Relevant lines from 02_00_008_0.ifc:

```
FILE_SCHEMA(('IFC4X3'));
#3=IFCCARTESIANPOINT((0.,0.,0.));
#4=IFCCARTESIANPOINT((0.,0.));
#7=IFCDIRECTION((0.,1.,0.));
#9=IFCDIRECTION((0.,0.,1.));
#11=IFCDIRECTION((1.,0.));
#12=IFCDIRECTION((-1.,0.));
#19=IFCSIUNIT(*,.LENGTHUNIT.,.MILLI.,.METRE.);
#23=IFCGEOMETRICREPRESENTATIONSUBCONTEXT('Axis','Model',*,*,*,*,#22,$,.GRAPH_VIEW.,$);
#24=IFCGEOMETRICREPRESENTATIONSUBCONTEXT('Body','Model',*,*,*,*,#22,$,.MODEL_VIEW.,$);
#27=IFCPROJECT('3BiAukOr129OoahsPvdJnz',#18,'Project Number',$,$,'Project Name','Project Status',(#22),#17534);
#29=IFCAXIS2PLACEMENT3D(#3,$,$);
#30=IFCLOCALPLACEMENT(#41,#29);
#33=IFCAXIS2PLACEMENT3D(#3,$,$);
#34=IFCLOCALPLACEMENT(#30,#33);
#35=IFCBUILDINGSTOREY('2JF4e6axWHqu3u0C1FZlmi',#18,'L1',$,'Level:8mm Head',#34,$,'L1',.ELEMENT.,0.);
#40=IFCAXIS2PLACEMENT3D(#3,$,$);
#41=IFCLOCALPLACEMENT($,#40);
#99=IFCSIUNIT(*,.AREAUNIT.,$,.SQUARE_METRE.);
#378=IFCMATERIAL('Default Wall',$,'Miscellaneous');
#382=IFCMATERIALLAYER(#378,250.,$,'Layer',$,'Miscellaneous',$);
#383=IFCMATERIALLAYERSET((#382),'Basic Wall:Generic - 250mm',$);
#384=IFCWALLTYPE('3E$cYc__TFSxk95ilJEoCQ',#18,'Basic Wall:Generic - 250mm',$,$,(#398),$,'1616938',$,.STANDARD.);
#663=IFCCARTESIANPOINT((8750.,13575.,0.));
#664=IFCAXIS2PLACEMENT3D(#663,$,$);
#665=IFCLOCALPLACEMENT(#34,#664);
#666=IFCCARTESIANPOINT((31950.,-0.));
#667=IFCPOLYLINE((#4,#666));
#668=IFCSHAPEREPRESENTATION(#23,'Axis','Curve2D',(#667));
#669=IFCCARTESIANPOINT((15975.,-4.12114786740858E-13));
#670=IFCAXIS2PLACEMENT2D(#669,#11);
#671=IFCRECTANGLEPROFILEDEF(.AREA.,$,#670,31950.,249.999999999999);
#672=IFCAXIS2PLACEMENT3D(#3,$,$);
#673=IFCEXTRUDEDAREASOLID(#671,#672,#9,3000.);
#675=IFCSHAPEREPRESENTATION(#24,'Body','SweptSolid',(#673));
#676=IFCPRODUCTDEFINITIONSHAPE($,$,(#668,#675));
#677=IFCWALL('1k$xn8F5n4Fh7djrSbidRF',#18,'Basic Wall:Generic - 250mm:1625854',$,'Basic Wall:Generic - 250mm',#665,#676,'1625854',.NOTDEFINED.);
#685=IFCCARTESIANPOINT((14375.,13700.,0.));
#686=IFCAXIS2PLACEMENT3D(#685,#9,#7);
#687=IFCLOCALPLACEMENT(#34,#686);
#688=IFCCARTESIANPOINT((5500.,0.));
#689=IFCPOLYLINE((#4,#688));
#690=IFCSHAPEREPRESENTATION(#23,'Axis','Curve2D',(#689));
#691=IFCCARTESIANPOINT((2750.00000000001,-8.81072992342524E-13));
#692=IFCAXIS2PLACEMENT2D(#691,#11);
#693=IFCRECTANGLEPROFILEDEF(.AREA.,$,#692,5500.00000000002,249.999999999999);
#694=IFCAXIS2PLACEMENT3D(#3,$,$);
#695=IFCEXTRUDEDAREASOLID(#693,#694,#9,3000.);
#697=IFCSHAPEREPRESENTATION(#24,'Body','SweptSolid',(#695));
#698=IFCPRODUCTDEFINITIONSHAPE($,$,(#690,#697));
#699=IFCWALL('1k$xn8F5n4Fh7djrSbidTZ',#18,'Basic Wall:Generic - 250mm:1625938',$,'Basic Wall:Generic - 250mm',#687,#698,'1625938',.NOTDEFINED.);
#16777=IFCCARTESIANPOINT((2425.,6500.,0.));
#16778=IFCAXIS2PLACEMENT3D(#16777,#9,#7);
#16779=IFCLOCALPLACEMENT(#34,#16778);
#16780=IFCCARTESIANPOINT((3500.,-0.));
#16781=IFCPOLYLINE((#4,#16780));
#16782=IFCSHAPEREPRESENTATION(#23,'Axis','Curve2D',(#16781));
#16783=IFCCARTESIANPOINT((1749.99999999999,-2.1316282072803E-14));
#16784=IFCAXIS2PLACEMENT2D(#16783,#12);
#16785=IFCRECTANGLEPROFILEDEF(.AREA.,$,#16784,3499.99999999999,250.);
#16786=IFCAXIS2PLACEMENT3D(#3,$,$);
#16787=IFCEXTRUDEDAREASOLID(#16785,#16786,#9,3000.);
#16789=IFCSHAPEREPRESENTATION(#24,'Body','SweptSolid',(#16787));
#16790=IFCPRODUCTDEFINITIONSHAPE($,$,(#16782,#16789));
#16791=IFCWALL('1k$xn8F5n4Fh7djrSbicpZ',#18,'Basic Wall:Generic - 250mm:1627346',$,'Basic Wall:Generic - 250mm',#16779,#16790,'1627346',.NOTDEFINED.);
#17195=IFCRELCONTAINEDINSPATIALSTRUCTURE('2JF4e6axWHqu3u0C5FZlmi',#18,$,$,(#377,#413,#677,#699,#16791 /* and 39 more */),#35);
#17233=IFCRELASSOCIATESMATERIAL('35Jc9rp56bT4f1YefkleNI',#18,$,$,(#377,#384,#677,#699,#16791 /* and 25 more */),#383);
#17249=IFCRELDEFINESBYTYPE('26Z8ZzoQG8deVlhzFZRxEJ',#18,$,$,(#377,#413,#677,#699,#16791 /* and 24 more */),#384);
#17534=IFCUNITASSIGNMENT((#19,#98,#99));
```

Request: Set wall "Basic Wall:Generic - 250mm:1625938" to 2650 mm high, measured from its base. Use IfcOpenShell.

```python
import ifcopenshell
import ifcopenshell.geom
import ifcopenshell.util.representation
import ifcopenshell.util.shape

model = ifcopenshell.open("02_00_008_0.ifc")
settings = ifcopenshell.geom.settings()


def volume(element):
    """Net volume in cubic metres, openings subtracted."""
    shape = ifcopenshell.geom.create_shape(settings, element)
    return ifcopenshell.util.shape.get_volume(shape.geometry)


wall = model.by_guid("1k$xn8F5n4Fh7djrSbidTZ")
before = volume(wall)

body = ifcopenshell.util.representation.get_representation(wall, "Model", "Body")
solid = body.Items[0]
old_height = solid.Depth
solid.Depth = 2650.0
after = volume(wall)

print(f"height {old_height:g} -> {solid.Depth:g}, volume {before:.3f} -> {after:.3f} m3")

model.write("02_00_008_0_rev.ifc")
```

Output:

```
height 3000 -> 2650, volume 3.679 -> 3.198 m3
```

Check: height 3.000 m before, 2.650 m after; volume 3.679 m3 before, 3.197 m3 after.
